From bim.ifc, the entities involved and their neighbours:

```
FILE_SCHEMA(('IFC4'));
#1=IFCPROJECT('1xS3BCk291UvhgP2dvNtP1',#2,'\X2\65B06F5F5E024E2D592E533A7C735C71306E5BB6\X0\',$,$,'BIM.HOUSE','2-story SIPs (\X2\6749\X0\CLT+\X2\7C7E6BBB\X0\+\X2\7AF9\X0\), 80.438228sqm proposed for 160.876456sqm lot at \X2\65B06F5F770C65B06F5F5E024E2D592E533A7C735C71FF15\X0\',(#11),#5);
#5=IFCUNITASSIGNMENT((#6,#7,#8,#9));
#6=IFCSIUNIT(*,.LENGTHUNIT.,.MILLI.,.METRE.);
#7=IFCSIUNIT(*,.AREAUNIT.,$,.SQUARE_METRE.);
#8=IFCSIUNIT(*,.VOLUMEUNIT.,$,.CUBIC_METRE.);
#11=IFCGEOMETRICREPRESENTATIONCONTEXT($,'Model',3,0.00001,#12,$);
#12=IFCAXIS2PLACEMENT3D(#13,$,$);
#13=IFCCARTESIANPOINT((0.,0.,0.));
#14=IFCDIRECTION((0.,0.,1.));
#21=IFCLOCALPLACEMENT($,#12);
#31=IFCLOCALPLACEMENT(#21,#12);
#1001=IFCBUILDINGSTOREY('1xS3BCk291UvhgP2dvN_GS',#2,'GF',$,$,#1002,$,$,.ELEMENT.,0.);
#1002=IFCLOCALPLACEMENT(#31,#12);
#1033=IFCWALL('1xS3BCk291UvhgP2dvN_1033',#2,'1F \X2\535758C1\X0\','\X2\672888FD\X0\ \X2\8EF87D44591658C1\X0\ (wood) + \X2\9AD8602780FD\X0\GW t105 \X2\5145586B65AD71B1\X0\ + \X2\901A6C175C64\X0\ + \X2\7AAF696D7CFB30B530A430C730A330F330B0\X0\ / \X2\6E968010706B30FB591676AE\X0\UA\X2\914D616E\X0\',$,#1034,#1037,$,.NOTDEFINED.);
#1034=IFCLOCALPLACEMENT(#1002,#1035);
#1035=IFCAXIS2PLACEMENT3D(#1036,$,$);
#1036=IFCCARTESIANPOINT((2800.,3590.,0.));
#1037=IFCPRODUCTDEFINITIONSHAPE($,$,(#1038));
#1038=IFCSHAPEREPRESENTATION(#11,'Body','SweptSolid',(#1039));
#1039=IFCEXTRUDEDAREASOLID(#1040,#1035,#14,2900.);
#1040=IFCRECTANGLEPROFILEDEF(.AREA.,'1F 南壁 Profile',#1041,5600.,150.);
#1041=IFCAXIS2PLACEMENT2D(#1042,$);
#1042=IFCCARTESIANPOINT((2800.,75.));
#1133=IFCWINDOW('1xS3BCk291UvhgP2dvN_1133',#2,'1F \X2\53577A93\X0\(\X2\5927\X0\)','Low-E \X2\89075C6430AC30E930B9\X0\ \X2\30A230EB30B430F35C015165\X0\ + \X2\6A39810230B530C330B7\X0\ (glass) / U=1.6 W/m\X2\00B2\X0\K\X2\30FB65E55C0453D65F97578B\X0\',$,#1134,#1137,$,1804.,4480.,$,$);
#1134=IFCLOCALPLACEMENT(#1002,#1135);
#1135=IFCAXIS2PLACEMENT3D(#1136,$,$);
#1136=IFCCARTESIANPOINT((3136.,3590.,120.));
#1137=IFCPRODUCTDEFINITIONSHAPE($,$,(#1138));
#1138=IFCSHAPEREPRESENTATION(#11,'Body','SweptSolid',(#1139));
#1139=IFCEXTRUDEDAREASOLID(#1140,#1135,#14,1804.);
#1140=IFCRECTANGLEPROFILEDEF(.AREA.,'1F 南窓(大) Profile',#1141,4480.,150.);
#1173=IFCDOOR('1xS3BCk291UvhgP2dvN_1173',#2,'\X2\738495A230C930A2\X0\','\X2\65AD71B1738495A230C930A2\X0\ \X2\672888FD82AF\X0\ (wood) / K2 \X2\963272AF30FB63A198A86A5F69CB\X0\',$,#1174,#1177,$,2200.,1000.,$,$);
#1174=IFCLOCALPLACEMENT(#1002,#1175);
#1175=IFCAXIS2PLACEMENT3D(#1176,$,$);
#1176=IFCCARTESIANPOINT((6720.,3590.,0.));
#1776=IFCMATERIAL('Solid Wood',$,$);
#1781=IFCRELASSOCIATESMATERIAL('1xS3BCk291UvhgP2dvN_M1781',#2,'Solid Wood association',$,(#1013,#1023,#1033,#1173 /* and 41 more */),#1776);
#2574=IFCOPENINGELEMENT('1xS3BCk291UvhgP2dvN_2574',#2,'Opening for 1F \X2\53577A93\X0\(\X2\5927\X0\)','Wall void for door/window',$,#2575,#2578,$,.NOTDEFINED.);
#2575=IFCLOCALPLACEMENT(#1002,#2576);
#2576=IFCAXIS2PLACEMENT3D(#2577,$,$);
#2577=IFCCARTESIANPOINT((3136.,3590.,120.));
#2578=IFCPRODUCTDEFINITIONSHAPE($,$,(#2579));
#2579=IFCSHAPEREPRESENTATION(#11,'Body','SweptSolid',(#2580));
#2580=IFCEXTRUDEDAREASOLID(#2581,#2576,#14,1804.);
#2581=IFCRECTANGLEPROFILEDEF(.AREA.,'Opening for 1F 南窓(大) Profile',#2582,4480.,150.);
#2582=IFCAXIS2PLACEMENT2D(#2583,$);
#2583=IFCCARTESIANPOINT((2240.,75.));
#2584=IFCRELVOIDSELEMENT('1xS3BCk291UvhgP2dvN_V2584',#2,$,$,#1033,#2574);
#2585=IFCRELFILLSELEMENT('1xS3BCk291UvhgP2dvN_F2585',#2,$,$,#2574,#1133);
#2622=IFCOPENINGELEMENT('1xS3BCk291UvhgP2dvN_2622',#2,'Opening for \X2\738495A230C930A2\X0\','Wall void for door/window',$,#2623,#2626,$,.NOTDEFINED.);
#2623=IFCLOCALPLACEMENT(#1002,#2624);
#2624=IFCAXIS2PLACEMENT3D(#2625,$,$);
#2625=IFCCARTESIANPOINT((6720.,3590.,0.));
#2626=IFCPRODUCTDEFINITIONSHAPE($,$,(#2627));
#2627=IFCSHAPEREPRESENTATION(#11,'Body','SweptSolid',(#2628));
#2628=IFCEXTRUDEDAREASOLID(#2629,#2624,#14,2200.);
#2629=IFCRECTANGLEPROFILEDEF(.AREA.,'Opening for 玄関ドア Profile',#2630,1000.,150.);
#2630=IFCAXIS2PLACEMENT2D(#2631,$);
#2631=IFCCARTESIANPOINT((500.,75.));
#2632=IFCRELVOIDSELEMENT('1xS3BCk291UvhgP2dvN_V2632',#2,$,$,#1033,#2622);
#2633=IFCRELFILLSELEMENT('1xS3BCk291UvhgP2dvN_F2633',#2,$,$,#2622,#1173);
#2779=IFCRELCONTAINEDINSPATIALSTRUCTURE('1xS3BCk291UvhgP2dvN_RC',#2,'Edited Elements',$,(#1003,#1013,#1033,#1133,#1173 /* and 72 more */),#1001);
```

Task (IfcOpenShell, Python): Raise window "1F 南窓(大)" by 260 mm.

```python
import numpy as np
import ifcopenshell
import ifcopenshell.api.geometry
import ifcopenshell.util.placement
import ifcopenshell.util.unit

model = ifcopenshell.open("bim.ifc")
unit_scale = ifcopenshell.util.unit.calculate_unit_scale(model)

window = model.by_id(1133)
opening = window.FillsVoids[0].RelatingOpeningElement
dz = 0.26 / unit_scale

shift = np.array([0.0, 0.0, dz])
# The window is not placed relative to its opening, so move both.
for product in (opening, window):
    matrix = ifcopenshell.util.placement.get_local_placement(product.ObjectPlacement)
    matrix[:3, 3] += shift
    ifcopenshell.api.geometry.edit_object_placement(model, product=product, matrix=matrix, is_si=False)

print(f"moved by {dz * unit_scale:+.3f} m")

model.write("bim_updated.ifc")
```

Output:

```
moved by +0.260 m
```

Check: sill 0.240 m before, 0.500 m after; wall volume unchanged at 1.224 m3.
